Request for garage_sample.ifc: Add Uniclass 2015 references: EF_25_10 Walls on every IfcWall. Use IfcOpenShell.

First a look at what the model holds.

```python
import ifcopenshell

model = ifcopenshell.open("garage_sample.ifc")
print(model.schema)
print("classifications:", [c.Name for c in model.by_type("IfcClassification")])
for ifc_class in ("IfcDoor", "IfcRoof", "IfcStair", "IfcWall", "IfcWindow"):
    print(ifc_class, len(model.by_type(ifc_class)))
```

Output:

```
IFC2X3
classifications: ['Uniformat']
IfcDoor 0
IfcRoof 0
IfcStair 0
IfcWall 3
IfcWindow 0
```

```python
import ifcopenshell
import ifcopenshell.api.classification

model = ifcopenshell.open("garage_sample.ifc")

# IFC2X3 requires Source and Edition and has no link from the project to the system.
system = model.create_entity("IfcClassification", Source="NBS", Edition="2015", Name="Uniclass 2015")

codes = {
    "IfcWall": ("EF_25_10", "Walls"),
}
for ifc_class, (code, name) in codes.items():
    products = model.by_type(ifc_class)
    ifcopenshell.api.classification.add_reference(
        model, products=products, classification=system, identification=code, name=name
    )
    print(code, len(products))

model.write("garage_sample-out.ifc")
```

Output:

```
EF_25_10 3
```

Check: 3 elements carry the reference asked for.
